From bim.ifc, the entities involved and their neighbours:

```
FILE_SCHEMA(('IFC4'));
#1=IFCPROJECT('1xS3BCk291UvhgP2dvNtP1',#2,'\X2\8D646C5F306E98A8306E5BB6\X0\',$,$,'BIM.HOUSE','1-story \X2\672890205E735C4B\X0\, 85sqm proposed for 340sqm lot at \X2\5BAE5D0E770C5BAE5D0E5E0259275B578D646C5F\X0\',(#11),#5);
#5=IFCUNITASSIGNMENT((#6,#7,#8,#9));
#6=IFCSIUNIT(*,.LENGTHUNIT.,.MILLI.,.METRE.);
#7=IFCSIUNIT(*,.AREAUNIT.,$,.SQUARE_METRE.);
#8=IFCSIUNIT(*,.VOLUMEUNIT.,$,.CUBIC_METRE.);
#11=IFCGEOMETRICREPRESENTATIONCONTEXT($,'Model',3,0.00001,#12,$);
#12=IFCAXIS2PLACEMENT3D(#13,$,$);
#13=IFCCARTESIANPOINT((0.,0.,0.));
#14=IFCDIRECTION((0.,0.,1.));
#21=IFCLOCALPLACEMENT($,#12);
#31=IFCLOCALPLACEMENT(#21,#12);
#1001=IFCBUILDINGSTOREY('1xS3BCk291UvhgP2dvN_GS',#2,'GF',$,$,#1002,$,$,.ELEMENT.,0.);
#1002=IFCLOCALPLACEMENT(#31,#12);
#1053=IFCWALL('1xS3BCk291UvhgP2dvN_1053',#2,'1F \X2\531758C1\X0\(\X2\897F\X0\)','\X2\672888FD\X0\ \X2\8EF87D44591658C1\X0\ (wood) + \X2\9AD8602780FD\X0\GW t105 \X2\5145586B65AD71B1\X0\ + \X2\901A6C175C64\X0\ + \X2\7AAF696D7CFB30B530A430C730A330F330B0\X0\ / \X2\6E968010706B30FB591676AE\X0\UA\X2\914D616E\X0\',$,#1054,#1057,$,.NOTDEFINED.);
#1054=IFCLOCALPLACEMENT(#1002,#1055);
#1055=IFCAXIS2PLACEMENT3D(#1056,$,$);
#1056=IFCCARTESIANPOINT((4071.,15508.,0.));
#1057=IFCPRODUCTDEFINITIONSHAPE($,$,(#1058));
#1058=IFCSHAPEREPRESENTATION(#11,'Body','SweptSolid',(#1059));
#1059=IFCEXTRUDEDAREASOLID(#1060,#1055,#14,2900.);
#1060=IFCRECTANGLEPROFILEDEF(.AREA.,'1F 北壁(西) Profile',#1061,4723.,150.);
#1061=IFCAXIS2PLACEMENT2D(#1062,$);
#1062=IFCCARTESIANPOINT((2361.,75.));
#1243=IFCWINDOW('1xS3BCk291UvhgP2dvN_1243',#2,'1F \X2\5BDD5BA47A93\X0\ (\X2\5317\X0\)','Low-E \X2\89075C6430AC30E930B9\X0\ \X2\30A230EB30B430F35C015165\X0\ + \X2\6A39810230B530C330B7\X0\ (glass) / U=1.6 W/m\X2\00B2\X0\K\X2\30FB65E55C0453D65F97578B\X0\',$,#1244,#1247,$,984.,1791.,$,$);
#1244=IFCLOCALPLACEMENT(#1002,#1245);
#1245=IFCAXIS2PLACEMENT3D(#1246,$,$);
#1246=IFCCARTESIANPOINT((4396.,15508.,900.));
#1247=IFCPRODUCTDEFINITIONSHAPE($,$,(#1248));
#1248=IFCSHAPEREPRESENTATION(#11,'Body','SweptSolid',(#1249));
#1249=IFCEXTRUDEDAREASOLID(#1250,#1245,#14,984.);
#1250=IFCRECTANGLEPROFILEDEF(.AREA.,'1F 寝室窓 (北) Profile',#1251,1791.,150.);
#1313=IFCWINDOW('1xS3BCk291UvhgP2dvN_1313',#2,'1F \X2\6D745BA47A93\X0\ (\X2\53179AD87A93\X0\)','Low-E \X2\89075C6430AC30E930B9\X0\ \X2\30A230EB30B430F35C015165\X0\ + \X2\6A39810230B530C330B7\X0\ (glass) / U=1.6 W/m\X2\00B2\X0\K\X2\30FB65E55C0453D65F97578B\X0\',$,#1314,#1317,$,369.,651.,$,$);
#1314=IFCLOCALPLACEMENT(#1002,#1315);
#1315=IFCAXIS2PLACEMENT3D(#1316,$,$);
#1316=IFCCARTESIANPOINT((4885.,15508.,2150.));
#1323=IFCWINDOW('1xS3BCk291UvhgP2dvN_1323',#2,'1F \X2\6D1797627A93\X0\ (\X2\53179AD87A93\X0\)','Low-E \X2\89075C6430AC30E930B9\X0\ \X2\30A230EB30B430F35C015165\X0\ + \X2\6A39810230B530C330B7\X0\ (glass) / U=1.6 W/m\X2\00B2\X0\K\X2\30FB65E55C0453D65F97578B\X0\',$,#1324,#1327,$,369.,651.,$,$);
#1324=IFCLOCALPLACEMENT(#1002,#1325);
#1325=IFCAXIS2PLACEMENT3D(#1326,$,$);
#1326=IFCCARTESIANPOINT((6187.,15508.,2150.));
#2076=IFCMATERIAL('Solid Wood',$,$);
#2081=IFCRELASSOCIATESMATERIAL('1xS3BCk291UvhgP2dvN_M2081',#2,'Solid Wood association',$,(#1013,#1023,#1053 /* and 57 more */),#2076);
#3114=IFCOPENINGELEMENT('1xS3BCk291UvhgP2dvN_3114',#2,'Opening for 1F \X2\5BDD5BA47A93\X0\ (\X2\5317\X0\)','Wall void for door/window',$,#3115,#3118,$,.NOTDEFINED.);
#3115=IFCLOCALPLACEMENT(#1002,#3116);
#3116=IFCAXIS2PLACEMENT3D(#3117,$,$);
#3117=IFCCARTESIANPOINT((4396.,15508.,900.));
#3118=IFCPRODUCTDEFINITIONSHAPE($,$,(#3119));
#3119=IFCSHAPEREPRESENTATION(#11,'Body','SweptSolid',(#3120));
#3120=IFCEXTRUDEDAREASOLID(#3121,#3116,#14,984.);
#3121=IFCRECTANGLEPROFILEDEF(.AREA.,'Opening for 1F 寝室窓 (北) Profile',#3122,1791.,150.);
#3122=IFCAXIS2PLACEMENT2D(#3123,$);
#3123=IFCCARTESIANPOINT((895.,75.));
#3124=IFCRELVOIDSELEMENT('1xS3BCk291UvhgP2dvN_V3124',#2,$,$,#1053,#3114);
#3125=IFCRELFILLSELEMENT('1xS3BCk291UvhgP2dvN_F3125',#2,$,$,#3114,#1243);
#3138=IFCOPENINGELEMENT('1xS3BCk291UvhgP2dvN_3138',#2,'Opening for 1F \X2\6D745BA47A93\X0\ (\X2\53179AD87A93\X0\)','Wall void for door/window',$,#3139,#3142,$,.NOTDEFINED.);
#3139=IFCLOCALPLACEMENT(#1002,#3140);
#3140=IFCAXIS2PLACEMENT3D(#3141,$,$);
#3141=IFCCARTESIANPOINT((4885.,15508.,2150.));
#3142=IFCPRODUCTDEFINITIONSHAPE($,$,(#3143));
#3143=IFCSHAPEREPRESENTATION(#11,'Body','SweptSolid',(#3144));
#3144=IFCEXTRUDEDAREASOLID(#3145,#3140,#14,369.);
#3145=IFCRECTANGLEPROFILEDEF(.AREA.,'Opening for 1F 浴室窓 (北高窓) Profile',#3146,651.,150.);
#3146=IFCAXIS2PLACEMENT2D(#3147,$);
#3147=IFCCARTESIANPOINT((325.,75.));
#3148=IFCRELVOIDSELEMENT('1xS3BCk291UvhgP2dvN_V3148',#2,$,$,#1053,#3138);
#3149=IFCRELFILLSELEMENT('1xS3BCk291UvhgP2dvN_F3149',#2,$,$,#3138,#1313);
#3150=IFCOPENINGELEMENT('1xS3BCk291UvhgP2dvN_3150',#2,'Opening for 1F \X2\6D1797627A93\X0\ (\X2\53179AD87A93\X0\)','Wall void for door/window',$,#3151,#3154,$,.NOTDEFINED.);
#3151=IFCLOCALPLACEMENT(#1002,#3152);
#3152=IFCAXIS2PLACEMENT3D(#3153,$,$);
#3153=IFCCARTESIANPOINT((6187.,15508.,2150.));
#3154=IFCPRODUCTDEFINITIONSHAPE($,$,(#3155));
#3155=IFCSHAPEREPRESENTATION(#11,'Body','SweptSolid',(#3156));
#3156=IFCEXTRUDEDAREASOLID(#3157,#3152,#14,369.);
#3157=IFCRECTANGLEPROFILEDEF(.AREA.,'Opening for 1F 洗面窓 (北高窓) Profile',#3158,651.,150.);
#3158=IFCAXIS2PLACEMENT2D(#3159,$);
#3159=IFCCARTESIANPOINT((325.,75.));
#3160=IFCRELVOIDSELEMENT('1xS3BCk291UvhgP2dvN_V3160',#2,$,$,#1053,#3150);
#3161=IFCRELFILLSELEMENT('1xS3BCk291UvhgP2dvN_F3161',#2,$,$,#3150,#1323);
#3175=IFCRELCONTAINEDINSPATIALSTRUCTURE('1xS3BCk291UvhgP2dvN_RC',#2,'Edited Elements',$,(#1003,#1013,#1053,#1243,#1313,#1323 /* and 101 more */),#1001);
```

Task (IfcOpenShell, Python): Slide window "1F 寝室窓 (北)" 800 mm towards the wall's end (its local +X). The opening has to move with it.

```python
import ifcopenshell
import ifcopenshell.api.geometry
import ifcopenshell.util.placement
import ifcopenshell.util.unit

model = ifcopenshell.open("bim.ifc")
unit_scale = ifcopenshell.util.unit.calculate_unit_scale(model)

window = model.by_guid("1xS3BCk291UvhgP2dvN_1243")
opening = window.FillsVoids[0].RelatingOpeningElement
wall = opening.VoidsElements[0].RelatingBuildingElement

wall_matrix = ifcopenshell.util.placement.get_local_placement(wall.ObjectPlacement)
shift = wall_matrix[:3, 0] * 0.8 / unit_scale
before = ifcopenshell.util.placement.get_local_placement(window.ObjectPlacement)[:3, 3].copy()

# The window is not placed relative to its opening, so move both.
for product in (opening, window):
    matrix = ifcopenshell.util.placement.get_local_placement(product.ObjectPlacement)
    matrix[:3, 3] += shift
    ifcopenshell.api.geometry.edit_object_placement(model, product=product, matrix=matrix, is_si=False)

after = ifcopenshell.util.placement.get_local_placement(window.ObjectPlacement)[:3, 3]
print("window moved by", (after - before).round(3) + 0.0)

model.write("bim_updated.ifc")
```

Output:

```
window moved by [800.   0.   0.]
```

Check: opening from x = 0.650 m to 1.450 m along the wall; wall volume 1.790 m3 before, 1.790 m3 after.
